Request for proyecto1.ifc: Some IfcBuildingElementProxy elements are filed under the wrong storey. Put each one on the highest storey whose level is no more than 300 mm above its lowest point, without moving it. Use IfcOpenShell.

First a look at what the model holds.

```python
import ifcopenshell
import ifcopenshell.util.element
import ifcopenshell.util.placement

model = ifcopenshell.open("proyecto1.ifc")
print(model.schema)
for storey in model.by_type("IfcBuildingStorey"):
    level = ifcopenshell.util.placement.get_storey_elevation(storey)
    count = sum(e.is_a("IfcBuildingElementProxy") for e in ifcopenshell.util.element.get_contained(storey))
    print(storey.id(), storey.Name, round(level, 3), count, sep=" | ")
```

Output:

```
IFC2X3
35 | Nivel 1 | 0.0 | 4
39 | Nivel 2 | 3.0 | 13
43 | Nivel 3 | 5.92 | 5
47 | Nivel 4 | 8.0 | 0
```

```python
import ifcopenshell
import ifcopenshell.api.spatial
import ifcopenshell.geom
import ifcopenshell.util.element
import ifcopenshell.util.placement
import ifcopenshell.util.shape
import ifcopenshell.util.unit

model = ifcopenshell.open("proyecto1.ifc")
unit_scale = ifcopenshell.util.unit.calculate_unit_scale(model)
settings = ifcopenshell.geom.settings()

levels = sorted(
    ((ifcopenshell.util.placement.get_storey_elevation(s) * unit_scale, s) for s in model.by_type("IfcBuildingStorey")),
    key=lambda pair: pair[0],
)

for e in model.by_type("IfcBuildingElementProxy"):
    current = e.ContainedInStructure[0].RelatingStructure if e.ContainedInStructure else None
    if current is None or not current.is_a("IfcBuildingStorey"):
        continue
    shape = ifcopenshell.geom.create_shape(settings, e)
    bottom = ifcopenshell.util.shape.get_shape_bottom_elevation(shape, shape.geometry)
    below = [s for level, s in levels if level <= bottom + 0.3]
    storey = below[-1] if below else levels[0][1]
    if storey != current:
        # assign_container keeps the world position.
        ifcopenshell.api.spatial.assign_container(model, products=[e], relating_structure=storey)
        print(e.id(), current.Name, "->", storey.Name)

model.write("proyecto1_edited.ifc")
```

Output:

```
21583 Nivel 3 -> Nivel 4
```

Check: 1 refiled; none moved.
